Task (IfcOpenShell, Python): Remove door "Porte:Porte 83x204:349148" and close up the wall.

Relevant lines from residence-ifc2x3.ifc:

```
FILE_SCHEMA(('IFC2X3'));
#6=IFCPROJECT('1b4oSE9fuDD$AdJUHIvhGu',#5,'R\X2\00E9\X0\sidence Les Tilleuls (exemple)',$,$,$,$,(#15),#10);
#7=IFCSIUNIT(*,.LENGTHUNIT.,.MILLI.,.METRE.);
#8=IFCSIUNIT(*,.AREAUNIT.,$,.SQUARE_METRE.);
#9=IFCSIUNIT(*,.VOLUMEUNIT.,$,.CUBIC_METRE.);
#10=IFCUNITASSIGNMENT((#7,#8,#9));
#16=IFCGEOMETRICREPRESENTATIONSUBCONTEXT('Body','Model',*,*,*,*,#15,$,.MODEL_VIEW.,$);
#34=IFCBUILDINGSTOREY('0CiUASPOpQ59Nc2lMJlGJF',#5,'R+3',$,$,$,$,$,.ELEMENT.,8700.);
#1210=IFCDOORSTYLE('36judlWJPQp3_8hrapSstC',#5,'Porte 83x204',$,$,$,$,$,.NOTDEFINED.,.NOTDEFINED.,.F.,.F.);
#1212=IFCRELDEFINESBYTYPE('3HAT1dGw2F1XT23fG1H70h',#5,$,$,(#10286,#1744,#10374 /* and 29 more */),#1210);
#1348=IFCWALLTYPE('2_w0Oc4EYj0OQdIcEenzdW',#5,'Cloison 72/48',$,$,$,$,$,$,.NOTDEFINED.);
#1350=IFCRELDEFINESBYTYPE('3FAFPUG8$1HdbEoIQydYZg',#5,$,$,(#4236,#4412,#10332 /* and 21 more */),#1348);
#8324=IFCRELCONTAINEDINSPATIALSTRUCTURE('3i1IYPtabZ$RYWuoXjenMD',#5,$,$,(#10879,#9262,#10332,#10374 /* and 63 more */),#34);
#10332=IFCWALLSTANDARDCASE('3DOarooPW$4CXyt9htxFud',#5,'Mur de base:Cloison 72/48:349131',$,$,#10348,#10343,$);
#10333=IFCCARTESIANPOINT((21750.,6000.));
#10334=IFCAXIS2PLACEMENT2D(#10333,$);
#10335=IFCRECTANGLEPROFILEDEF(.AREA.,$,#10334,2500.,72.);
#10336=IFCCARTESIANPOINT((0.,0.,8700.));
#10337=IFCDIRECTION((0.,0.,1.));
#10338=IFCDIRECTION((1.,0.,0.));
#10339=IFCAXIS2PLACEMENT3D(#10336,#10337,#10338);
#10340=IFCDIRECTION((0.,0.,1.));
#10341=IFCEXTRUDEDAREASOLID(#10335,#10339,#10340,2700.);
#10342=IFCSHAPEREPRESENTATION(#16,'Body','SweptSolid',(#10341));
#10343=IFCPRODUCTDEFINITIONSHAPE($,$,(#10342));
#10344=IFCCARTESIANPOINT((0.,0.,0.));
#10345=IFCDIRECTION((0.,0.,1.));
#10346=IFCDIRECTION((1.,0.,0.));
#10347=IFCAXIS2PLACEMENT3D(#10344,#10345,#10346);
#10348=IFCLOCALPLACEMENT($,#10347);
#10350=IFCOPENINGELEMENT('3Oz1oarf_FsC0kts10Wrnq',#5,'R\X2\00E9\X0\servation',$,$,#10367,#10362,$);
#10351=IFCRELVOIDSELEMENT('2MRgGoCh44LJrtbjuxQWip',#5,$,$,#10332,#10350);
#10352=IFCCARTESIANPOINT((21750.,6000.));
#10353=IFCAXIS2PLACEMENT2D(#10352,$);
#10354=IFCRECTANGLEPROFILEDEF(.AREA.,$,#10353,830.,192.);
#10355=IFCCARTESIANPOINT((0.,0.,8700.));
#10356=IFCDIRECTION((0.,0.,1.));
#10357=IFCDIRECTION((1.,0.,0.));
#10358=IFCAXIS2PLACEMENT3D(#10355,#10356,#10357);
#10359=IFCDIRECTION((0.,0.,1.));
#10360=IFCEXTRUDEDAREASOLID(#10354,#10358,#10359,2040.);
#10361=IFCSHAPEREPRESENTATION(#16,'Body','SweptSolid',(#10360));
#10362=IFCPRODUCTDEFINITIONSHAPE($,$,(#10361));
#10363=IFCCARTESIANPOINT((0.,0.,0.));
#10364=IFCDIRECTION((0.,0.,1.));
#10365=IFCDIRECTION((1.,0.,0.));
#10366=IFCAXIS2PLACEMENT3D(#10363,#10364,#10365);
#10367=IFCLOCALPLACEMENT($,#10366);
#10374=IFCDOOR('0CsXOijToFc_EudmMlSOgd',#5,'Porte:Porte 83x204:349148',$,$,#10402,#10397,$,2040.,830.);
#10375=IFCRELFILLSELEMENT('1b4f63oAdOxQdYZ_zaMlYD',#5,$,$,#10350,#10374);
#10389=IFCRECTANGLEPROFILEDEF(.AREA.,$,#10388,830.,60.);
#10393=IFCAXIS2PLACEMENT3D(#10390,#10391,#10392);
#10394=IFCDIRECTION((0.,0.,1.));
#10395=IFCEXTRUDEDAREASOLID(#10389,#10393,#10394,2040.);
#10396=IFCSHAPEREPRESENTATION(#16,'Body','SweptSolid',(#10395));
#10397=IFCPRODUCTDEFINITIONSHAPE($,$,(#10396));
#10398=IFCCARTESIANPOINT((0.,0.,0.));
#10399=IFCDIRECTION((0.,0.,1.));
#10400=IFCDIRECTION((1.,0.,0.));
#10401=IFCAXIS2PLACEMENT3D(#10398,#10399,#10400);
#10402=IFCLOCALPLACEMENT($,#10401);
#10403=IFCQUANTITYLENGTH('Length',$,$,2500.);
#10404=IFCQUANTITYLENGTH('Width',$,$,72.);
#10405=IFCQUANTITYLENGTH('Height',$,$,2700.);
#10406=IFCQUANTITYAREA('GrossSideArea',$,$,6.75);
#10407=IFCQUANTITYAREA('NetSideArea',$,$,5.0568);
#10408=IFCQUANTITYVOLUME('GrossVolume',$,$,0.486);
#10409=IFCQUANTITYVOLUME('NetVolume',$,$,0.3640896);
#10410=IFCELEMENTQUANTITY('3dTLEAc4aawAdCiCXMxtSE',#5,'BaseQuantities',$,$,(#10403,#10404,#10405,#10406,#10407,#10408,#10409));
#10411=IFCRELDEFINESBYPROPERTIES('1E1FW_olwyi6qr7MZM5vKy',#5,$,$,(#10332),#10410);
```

```python
import ifcopenshell
import ifcopenshell.api.feature
import ifcopenshell.api.pset
import ifcopenshell.api.root
import ifcopenshell.geom
import ifcopenshell.util.element
import ifcopenshell.util.shape
import ifcopenshell.util.unit

model = ifcopenshell.open("residence-ifc2x3.ifc")
area_scale = ifcopenshell.util.unit.calculate_unit_scale(model, "AREAUNIT")
volume_scale = ifcopenshell.util.unit.calculate_unit_scale(model, "VOLUMEUNIT")
settings = ifcopenshell.geom.settings()


def volume(element):
    """Net volume in cubic metres, openings subtracted."""
    shape = ifcopenshell.geom.create_shape(settings, element)
    return ifcopenshell.util.shape.get_volume(shape.geometry)


door = model.by_id(10374)
opening = door.FillsVoids[0].RelatingOpeningElement
wall = opening.VoidsElements[0].RelatingBuildingElement
before = volume(wall)

ifcopenshell.api.root.remove_product(model, product=door)
ifcopenshell.api.feature.remove_feature(model, feature=opening)

after = volume(wall)
thickness = 0.072  # wall thickness in metres

# Update the wall's stored quantities.
qto = model.by_id(ifcopenshell.util.element.get_pset(wall, "BaseQuantities", should_inherit=False)["id"])
ifcopenshell.api.pset.edit_qto(model, qto=qto, properties={
    "NetSideArea": after / thickness / area_scale,
    "NetVolume": after / volume_scale,
})

print(f"wall volume {before:.3f} -> {after:.3f} m3")

model.write("residence-ifc2x3_edited.ifc")
```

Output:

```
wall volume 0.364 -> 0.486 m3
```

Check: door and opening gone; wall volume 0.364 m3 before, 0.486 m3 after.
